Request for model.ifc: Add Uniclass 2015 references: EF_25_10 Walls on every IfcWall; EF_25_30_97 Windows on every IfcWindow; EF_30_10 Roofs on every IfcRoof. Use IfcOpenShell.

First a look at what the model holds.

```python
import ifcopenshell

model = ifcopenshell.open("model.ifc")
print(model.schema)
print("classifications:", [c.Name for c in model.by_type("IfcClassification")])
for ifc_class in ("IfcDoor", "IfcRoof", "IfcStair", "IfcWall", "IfcWindow"):
    print(ifc_class, len(model.by_type(ifc_class)))
```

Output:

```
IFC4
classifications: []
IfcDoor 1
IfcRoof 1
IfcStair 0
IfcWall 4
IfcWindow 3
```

```python
import ifcopenshell
import ifcopenshell.api.classification

model = ifcopenshell.open("model.ifc")

system = ifcopenshell.api.classification.add_classification(model, classification="Uniclass 2015")

codes = {
    "IfcWall": ("EF_25_10", "Walls"),
    "IfcWindow": ("EF_25_30_97", "Windows"),
    "IfcRoof": ("EF_30_10", "Roofs"),
}
for ifc_class, (code, name) in codes.items():
    products = model.by_type(ifc_class)
    ifcopenshell.api.classification.add_reference(
        model, products=products, classification=system, identification=code, name=name
    )
    print(code, len(products))

model.write("model-out.ifc")
```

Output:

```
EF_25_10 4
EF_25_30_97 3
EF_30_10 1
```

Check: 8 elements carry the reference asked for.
